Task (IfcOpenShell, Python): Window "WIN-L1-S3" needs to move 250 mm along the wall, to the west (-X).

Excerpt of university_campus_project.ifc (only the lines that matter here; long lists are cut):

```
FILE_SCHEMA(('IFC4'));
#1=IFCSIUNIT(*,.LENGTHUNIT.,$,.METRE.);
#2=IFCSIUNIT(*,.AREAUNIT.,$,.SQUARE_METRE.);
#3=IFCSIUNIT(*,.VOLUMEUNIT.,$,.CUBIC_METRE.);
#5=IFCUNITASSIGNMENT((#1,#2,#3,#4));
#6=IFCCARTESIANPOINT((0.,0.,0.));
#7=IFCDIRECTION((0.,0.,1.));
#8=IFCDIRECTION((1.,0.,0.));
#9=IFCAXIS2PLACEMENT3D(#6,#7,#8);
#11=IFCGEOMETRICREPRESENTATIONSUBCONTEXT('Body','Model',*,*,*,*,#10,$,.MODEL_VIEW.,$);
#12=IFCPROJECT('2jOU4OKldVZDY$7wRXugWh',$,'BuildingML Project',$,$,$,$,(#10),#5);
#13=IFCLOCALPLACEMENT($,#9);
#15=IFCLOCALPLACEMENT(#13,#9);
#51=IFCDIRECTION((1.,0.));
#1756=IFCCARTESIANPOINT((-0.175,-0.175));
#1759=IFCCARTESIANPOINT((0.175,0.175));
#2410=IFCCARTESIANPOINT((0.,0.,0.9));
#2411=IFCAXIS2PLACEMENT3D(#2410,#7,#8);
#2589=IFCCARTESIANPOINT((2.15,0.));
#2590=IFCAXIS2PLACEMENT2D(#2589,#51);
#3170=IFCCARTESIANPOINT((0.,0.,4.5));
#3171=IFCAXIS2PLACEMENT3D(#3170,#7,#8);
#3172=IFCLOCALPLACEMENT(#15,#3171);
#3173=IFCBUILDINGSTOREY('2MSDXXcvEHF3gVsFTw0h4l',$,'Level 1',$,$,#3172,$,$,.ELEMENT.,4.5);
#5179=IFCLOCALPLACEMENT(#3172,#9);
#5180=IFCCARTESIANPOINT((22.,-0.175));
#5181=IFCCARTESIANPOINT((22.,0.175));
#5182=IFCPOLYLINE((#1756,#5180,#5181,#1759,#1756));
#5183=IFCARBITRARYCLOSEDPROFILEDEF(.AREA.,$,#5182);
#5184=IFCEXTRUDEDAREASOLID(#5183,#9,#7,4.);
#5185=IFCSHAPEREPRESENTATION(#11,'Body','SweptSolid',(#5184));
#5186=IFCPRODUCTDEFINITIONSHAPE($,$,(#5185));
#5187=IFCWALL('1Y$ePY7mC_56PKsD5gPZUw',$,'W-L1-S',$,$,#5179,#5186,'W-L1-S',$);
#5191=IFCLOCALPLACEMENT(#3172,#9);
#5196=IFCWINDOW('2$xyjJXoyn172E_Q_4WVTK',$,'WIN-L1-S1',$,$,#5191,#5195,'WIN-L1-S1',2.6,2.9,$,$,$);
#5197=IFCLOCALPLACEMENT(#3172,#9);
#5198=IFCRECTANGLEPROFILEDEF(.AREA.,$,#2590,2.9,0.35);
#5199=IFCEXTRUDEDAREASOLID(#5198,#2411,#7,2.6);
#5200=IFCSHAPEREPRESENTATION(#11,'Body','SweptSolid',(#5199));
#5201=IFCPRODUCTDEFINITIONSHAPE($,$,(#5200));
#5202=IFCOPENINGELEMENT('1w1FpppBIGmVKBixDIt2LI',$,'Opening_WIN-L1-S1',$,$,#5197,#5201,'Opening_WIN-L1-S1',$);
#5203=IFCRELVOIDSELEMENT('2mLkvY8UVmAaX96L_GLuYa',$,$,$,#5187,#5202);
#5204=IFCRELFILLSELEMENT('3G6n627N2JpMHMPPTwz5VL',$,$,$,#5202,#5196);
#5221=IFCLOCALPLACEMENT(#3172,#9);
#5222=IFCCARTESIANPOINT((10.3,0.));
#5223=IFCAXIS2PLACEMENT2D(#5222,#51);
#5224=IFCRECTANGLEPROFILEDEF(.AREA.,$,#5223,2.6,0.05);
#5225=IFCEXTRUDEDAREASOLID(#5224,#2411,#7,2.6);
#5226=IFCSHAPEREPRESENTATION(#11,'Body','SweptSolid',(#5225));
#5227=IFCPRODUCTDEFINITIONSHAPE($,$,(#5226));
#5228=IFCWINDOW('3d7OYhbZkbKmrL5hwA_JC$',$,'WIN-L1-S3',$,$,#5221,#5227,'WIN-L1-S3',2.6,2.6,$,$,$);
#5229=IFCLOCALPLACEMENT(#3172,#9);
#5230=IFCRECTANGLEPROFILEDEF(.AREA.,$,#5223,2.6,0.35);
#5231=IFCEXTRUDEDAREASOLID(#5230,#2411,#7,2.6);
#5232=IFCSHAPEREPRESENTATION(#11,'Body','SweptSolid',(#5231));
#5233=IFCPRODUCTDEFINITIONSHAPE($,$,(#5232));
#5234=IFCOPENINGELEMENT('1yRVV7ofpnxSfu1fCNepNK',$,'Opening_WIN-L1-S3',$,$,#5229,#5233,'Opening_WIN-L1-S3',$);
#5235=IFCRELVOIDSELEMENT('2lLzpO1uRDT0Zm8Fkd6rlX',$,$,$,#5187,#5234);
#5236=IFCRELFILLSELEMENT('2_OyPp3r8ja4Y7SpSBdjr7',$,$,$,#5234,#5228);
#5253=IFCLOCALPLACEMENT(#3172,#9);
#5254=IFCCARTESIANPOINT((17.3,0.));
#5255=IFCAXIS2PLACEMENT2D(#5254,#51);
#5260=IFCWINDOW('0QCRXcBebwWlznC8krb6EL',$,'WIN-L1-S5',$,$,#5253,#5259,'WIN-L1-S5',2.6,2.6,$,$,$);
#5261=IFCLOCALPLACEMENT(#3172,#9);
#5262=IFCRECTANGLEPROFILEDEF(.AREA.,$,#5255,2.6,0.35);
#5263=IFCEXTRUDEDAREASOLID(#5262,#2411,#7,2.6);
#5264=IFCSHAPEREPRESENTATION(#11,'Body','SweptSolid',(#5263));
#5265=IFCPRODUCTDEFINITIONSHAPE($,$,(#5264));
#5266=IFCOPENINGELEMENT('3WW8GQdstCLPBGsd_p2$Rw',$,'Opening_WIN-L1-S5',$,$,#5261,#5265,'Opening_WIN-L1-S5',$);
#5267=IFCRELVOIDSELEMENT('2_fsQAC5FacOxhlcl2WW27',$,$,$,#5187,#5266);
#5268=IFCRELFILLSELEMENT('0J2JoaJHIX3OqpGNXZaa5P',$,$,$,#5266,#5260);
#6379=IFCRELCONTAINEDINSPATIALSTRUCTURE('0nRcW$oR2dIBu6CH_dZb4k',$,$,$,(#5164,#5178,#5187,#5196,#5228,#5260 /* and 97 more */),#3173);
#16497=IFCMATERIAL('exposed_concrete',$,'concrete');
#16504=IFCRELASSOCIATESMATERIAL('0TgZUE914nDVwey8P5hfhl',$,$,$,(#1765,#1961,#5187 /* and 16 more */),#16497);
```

```python
import ifcopenshell
import ifcopenshell.api.geometry
import ifcopenshell.util.placement
import ifcopenshell.util.unit

model = ifcopenshell.open("university_campus_project.ifc")
unit_scale = ifcopenshell.util.unit.calculate_unit_scale(model)

window = model.by_id(5228)
opening = window.FillsVoids[0].RelatingOpeningElement
wall = opening.VoidsElements[0].RelatingBuildingElement

wall_matrix = ifcopenshell.util.placement.get_local_placement(wall.ObjectPlacement)
shift = wall_matrix[:3, 0] * -0.25 / unit_scale
before = ifcopenshell.util.placement.get_local_placement(window.ObjectPlacement)[:3, 3].copy()

# The window is not placed relative to its opening, so move both.
for product in (opening, window):
    matrix = ifcopenshell.util.placement.get_local_placement(product.ObjectPlacement)
    matrix[:3, 3] += shift
    ifcopenshell.api.geometry.edit_object_placement(model, product=product, matrix=matrix, is_si=False)

after = ifcopenshell.util.placement.get_local_placement(window.ObjectPlacement)[:3, 3]
print("window moved by", (after - before).round(3) + 0.0)

model.write("university_campus_project_updated.ifc")
```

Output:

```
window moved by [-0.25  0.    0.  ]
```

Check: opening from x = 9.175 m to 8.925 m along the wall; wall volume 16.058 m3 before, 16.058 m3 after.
